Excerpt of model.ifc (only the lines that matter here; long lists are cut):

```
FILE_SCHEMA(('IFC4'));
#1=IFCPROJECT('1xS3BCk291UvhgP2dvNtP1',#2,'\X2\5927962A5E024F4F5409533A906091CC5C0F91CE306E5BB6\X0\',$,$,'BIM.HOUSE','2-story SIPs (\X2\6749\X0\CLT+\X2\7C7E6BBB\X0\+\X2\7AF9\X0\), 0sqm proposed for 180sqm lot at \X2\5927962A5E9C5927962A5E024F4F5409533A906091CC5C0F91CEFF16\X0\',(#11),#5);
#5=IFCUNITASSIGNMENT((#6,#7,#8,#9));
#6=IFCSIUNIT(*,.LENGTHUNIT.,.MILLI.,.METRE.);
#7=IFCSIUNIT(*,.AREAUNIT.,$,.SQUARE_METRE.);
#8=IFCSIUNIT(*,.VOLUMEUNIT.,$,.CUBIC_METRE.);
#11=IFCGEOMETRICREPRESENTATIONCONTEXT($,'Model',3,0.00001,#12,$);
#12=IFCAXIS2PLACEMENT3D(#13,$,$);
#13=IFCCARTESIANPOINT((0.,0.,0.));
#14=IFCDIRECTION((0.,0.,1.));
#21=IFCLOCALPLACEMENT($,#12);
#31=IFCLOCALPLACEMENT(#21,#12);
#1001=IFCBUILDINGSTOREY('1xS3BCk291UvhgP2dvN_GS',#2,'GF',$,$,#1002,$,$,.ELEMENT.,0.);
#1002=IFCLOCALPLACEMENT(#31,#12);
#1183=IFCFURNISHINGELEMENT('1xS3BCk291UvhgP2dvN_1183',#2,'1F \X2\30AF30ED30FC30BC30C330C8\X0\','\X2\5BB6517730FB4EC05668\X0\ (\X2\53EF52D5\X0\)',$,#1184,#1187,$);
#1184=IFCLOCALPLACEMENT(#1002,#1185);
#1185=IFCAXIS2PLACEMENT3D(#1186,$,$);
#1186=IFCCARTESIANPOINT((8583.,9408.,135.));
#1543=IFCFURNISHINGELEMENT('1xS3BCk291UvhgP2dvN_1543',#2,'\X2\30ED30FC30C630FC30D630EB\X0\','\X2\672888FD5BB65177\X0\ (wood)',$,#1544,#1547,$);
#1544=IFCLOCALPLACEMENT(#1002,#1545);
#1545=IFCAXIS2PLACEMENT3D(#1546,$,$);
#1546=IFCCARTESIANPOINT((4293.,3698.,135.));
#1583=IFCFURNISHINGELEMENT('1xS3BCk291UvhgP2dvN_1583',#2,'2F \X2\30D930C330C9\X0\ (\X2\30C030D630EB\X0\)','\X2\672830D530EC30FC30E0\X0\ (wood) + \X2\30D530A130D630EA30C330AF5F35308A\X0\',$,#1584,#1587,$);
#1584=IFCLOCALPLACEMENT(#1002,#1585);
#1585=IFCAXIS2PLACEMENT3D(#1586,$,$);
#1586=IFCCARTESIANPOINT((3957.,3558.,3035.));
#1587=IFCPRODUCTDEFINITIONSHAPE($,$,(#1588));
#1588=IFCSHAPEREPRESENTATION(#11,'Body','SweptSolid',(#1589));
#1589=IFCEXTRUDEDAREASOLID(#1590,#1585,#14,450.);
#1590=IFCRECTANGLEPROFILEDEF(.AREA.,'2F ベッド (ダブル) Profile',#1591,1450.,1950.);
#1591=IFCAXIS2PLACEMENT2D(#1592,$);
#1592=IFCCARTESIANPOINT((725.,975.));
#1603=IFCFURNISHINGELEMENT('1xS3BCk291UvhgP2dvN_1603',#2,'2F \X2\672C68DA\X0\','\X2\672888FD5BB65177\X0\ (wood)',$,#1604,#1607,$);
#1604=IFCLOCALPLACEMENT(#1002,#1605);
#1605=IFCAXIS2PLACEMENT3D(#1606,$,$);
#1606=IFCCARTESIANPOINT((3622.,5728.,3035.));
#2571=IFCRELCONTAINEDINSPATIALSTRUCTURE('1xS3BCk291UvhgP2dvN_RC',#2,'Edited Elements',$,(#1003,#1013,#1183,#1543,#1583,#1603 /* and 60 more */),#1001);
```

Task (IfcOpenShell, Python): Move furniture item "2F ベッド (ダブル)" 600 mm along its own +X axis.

```python
import ifcopenshell
import ifcopenshell.api.geometry
import ifcopenshell.util.placement
import ifcopenshell.util.unit

model = ifcopenshell.open("model.ifc")
unit_scale = ifcopenshell.util.unit.calculate_unit_scale(model)

item = model.by_id(1583)
matrix = ifcopenshell.util.placement.get_local_placement(item.ObjectPlacement)
matrix[:3, 3] += matrix[:3, 0] * 0.6 / unit_scale
ifcopenshell.api.geometry.edit_object_placement(model, product=item, matrix=matrix, is_si=False)

print(ifcopenshell.util.placement.get_local_placement(item.ObjectPlacement).round(3) + 0.0)

model.write("model_updated.ifc")
```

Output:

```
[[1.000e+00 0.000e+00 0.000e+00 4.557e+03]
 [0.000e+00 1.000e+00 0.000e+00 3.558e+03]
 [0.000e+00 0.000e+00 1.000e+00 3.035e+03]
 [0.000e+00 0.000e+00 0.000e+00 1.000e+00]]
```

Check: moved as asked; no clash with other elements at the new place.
